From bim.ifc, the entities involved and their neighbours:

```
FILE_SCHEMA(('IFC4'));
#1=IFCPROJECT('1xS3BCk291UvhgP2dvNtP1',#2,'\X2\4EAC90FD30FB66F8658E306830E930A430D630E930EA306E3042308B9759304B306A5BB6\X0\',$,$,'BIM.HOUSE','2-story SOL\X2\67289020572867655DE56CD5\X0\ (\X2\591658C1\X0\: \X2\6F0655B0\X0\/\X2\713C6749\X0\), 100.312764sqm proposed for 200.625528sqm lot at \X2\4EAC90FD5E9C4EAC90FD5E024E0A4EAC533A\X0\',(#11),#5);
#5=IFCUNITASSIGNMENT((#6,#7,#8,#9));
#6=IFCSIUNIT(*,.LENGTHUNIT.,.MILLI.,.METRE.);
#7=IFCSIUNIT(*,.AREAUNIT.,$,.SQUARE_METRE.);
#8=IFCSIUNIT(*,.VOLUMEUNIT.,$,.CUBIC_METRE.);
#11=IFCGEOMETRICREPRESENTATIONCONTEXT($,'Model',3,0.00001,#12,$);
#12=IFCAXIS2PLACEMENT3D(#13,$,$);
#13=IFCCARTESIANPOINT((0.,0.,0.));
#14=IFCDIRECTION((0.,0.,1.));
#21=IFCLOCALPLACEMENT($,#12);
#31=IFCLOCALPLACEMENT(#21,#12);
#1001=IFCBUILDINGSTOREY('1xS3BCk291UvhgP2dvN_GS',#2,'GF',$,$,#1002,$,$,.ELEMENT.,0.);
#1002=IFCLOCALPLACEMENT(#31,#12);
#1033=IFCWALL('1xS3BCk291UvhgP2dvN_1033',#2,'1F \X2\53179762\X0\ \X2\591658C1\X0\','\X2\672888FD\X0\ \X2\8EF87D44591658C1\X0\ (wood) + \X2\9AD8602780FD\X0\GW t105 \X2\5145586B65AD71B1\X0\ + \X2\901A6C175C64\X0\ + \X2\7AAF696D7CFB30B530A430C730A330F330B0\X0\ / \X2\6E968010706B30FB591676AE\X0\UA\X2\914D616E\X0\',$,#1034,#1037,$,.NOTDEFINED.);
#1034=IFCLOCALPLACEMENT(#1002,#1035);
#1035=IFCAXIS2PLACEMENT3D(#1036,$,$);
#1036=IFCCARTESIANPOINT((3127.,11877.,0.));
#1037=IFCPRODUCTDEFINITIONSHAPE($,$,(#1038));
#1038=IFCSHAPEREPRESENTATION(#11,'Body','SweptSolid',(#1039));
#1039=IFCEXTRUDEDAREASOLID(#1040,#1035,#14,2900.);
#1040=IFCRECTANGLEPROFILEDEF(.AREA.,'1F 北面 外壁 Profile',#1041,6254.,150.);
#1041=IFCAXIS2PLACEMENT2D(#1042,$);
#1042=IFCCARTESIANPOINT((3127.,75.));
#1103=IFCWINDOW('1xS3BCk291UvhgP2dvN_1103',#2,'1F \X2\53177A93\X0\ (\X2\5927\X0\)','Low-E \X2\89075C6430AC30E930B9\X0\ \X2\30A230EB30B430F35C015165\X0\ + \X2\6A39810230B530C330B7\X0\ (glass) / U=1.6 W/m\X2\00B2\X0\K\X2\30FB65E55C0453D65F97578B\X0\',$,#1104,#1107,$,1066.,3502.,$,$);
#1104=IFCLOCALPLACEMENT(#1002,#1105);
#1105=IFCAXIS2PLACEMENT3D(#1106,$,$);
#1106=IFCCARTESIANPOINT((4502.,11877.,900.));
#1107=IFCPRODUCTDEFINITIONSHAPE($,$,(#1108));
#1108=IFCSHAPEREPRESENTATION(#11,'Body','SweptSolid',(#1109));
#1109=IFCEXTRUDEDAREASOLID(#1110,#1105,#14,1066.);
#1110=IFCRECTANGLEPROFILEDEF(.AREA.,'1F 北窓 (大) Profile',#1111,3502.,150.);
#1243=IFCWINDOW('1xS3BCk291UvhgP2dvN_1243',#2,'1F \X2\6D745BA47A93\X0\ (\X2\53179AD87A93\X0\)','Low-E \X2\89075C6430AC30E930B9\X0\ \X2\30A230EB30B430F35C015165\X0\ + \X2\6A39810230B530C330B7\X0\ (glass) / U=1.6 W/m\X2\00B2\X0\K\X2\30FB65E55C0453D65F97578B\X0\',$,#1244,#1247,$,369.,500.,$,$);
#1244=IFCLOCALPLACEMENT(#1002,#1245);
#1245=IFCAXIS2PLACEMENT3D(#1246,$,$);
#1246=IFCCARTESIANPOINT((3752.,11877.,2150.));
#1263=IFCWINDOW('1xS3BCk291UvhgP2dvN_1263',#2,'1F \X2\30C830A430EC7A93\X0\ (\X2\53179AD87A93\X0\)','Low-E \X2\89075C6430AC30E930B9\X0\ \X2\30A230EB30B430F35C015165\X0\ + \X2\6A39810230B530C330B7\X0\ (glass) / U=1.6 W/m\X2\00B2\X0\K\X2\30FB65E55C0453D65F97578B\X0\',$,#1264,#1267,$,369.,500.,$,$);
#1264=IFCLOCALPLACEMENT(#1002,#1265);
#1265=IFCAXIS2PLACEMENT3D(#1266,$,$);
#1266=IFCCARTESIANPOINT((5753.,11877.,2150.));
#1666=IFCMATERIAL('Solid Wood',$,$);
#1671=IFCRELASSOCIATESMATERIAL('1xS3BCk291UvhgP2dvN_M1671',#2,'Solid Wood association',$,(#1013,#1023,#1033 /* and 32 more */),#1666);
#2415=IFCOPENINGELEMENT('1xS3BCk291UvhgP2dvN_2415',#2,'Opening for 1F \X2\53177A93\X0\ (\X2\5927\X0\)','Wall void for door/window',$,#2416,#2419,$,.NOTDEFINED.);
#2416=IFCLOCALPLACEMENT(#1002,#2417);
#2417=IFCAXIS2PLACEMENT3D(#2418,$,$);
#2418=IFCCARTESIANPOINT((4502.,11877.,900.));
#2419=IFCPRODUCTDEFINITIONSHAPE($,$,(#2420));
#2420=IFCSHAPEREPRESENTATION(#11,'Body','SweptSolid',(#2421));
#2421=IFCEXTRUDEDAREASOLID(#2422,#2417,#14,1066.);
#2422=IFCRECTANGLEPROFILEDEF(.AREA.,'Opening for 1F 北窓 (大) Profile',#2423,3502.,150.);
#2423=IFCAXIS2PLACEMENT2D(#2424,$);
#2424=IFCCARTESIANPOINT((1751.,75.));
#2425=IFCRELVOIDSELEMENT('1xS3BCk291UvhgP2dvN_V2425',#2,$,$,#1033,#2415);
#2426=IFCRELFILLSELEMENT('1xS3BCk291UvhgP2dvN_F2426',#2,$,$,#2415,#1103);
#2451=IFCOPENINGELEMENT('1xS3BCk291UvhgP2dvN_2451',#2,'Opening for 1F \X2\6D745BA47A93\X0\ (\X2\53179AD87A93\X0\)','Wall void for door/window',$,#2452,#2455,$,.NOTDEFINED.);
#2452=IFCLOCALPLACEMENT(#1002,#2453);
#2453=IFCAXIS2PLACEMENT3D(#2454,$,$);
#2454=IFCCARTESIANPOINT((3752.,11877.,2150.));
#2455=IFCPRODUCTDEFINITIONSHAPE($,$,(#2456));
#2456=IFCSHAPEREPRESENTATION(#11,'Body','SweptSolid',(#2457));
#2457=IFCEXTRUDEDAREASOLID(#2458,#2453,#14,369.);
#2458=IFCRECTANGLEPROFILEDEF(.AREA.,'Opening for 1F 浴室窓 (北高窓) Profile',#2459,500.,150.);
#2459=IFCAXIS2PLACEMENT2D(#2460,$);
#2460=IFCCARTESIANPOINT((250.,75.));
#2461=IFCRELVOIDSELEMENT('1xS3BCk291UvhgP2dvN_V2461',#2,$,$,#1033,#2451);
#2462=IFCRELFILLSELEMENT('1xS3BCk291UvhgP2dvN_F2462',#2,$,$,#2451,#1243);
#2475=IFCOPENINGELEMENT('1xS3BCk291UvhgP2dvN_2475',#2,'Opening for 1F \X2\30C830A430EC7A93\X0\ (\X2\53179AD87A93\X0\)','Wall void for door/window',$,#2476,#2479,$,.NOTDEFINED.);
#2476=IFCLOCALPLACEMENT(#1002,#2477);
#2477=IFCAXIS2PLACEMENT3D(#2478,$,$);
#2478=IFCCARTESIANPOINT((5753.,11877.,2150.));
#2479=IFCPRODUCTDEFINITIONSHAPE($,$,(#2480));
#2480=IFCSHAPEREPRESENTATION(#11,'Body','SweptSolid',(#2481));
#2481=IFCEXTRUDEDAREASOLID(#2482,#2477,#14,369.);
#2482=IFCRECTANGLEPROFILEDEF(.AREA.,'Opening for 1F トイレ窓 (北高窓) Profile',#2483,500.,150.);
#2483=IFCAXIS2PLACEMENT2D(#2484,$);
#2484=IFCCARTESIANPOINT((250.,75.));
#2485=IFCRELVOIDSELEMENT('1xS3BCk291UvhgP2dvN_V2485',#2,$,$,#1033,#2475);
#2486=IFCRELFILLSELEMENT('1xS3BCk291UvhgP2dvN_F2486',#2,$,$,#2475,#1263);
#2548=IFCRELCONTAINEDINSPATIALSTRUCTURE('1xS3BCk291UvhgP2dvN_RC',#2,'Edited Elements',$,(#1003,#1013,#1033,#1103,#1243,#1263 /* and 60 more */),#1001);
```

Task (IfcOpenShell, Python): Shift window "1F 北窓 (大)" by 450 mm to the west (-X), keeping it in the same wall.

```python
import ifcopenshell
import ifcopenshell.api.geometry
import ifcopenshell.util.placement
import ifcopenshell.util.unit

model = ifcopenshell.open("bim.ifc")
unit_scale = ifcopenshell.util.unit.calculate_unit_scale(model)

window = model.by_id(1103)
opening = window.FillsVoids[0].RelatingOpeningElement
wall = opening.VoidsElements[0].RelatingBuildingElement

wall_matrix = ifcopenshell.util.placement.get_local_placement(wall.ObjectPlacement)
shift = wall_matrix[:3, 0] * -0.45 / unit_scale
before = ifcopenshell.util.placement.get_local_placement(window.ObjectPlacement)[:3, 3].copy()

# The window is not placed relative to its opening, so move both.
for product in (opening, window):
    matrix = ifcopenshell.util.placement.get_local_placement(product.ObjectPlacement)
    matrix[:3, 3] += shift
    ifcopenshell.api.geometry.edit_object_placement(model, product=product, matrix=matrix, is_si=False)

after = ifcopenshell.util.placement.get_local_placement(window.ObjectPlacement)[:3, 3]
print("window moved by", (after - before).round(3) + 0.0)

model.write("bim_updated.ifc")
```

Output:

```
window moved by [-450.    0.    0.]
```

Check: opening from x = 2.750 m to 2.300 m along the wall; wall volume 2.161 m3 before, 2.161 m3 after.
